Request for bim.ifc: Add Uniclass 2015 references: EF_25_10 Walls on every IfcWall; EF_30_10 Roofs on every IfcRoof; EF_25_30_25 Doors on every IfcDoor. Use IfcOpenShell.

First a look at what the model holds.

```python
import ifcopenshell

model = ifcopenshell.open("bim.ifc")
print(model.schema)
print("classifications:", [c.Name for c in model.by_type("IfcClassification")])
for ifc_class in ("IfcDoor", "IfcRoof", "IfcStair", "IfcWall", "IfcWindow"):
    print(ifc_class, len(model.by_type(ifc_class)))
```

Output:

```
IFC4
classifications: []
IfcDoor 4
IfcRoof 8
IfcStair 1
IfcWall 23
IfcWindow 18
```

```python
import ifcopenshell
import ifcopenshell.api.classification

model = ifcopenshell.open("bim.ifc")

system = ifcopenshell.api.classification.add_classification(model, classification="Uniclass 2015")

codes = {
    "IfcWall": ("EF_25_10", "Walls"),
    "IfcRoof": ("EF_30_10", "Roofs"),
    "IfcDoor": ("EF_25_30_25", "Doors"),
}
for ifc_class, (code, name) in codes.items():
    products = model.by_type(ifc_class)
    ifcopenshell.api.classification.add_reference(
        model, products=products, classification=system, identification=code, name=name
    )
    print(code, len(products))

model.write("bim_rev.ifc")
```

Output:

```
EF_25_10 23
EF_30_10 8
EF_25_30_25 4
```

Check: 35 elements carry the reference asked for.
